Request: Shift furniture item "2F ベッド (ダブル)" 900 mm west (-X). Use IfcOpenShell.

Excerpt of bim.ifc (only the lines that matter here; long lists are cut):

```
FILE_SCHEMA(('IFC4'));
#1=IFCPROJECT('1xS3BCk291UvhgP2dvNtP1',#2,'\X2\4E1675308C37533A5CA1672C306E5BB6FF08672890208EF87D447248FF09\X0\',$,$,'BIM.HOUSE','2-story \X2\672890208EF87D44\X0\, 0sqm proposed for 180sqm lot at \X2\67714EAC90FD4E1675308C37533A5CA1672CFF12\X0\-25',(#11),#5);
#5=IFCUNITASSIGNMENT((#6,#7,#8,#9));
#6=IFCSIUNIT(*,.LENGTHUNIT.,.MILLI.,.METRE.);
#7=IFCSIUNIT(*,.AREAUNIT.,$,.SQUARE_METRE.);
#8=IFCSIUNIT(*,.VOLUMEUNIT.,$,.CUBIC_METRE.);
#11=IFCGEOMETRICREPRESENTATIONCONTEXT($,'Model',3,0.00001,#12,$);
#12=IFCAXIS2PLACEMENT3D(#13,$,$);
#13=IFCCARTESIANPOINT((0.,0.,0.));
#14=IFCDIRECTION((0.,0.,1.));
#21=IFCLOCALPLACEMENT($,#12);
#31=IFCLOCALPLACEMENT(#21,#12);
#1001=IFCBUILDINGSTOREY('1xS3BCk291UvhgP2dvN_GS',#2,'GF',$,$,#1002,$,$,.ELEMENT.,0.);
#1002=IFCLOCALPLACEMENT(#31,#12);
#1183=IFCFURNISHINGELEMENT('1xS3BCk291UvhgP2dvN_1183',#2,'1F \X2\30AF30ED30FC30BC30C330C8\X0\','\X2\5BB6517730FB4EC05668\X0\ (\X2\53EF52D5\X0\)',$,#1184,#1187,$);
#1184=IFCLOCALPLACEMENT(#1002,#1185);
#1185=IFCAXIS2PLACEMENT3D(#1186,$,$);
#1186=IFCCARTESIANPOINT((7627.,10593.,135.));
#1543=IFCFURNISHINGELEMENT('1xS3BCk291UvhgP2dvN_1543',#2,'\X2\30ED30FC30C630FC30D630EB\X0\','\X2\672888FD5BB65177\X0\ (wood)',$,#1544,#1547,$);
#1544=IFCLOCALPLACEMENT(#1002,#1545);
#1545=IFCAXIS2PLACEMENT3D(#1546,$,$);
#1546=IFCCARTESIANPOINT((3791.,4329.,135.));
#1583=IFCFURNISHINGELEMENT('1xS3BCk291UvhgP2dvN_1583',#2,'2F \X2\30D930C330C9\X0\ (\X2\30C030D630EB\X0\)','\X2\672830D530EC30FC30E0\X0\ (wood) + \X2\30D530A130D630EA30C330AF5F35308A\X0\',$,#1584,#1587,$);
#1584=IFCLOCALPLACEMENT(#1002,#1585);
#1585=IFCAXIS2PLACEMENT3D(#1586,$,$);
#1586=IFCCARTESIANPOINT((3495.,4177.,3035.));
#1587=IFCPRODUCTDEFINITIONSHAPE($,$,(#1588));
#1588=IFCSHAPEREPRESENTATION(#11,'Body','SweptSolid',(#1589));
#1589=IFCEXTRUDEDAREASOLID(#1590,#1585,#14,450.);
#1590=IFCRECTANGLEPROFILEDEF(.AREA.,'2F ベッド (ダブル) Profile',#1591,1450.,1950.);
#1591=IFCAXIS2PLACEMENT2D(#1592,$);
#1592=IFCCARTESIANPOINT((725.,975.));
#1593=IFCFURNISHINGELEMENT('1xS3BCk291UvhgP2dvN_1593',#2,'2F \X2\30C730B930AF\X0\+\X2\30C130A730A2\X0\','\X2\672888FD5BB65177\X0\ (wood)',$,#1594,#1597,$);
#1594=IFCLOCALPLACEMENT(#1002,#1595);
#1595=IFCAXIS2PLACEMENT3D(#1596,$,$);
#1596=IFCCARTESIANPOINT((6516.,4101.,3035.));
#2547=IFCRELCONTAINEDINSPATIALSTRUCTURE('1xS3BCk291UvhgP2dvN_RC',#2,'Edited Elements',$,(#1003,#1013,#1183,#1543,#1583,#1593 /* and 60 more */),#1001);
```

```python
import ifcopenshell
import ifcopenshell.api.geometry
import ifcopenshell.util.placement
import ifcopenshell.util.unit

model = ifcopenshell.open("bim.ifc")
unit_scale = ifcopenshell.util.unit.calculate_unit_scale(model)

item = model.by_guid("1xS3BCk291UvhgP2dvN_1583")
matrix = ifcopenshell.util.placement.get_local_placement(item.ObjectPlacement)
matrix[0, 3] -= 0.9 / unit_scale
ifcopenshell.api.geometry.edit_object_placement(model, product=item, matrix=matrix, is_si=False)

print(ifcopenshell.util.placement.get_local_placement(item.ObjectPlacement).round(3) + 0.0)

model.write("bim_edited.ifc")
```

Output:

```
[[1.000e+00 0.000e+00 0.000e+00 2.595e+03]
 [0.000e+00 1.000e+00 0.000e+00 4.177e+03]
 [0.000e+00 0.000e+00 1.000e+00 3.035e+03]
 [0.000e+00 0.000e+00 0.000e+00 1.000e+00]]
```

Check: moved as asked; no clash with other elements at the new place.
